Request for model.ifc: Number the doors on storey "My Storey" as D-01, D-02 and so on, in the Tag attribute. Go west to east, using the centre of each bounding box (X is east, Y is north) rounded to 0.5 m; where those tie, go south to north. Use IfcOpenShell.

First a look at what the model holds.

```python
import ifcopenshell
import ifcopenshell.util.element
import ifcopenshell.util.placement

model = ifcopenshell.open("model.ifc")
print(model.schema)
storey = next(s for s in model.by_type("IfcBuildingStorey") if s.Name == "My Storey")
doors = [e for e in ifcopenshell.util.element.get_decomposition(storey) if e.is_a("IfcDoor")]
for e in sorted(doors, key=lambda e: e.id()):
    origin = ifcopenshell.util.placement.get_local_placement(e.ObjectPlacement)[:3, 3]
    print(e.id(), e.Tag, e.Name, origin.round(2) + 0.0, sep=" | ")
```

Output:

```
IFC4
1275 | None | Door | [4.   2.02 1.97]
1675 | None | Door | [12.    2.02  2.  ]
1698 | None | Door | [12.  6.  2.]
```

```python
import ifcopenshell
import ifcopenshell.geom
import ifcopenshell.util.element
import ifcopenshell.util.shape

model = ifcopenshell.open("model.ifc")
settings = ifcopenshell.geom.settings()
settings.set("use-world-coords", True)


def centre(element):
    shape = ifcopenshell.geom.create_shape(settings, element)
    return ifcopenshell.util.shape.get_bbox_centroid(shape.geometry)


storey = next(s for s in model.by_type("IfcBuildingStorey") if s.Name == "My Storey")
doors = [e for e in ifcopenshell.util.element.get_decomposition(storey) if e.is_a("IfcDoor")]

# Insertion points can sit at a corner or the storey origin, so sort by the geometry (in metres).
centres = {e: centre(e) for e in doors}
doors.sort(key=lambda e: (round(centres[e][0] / 0.5), centres[e][1]))

for i, e in enumerate(doors, start=1):
    number = f"D-{i:02d}"
    e.Tag = number
    print(e.id(), number)

model.write("model_edited.ifc")
```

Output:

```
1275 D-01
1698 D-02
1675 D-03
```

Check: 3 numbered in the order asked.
